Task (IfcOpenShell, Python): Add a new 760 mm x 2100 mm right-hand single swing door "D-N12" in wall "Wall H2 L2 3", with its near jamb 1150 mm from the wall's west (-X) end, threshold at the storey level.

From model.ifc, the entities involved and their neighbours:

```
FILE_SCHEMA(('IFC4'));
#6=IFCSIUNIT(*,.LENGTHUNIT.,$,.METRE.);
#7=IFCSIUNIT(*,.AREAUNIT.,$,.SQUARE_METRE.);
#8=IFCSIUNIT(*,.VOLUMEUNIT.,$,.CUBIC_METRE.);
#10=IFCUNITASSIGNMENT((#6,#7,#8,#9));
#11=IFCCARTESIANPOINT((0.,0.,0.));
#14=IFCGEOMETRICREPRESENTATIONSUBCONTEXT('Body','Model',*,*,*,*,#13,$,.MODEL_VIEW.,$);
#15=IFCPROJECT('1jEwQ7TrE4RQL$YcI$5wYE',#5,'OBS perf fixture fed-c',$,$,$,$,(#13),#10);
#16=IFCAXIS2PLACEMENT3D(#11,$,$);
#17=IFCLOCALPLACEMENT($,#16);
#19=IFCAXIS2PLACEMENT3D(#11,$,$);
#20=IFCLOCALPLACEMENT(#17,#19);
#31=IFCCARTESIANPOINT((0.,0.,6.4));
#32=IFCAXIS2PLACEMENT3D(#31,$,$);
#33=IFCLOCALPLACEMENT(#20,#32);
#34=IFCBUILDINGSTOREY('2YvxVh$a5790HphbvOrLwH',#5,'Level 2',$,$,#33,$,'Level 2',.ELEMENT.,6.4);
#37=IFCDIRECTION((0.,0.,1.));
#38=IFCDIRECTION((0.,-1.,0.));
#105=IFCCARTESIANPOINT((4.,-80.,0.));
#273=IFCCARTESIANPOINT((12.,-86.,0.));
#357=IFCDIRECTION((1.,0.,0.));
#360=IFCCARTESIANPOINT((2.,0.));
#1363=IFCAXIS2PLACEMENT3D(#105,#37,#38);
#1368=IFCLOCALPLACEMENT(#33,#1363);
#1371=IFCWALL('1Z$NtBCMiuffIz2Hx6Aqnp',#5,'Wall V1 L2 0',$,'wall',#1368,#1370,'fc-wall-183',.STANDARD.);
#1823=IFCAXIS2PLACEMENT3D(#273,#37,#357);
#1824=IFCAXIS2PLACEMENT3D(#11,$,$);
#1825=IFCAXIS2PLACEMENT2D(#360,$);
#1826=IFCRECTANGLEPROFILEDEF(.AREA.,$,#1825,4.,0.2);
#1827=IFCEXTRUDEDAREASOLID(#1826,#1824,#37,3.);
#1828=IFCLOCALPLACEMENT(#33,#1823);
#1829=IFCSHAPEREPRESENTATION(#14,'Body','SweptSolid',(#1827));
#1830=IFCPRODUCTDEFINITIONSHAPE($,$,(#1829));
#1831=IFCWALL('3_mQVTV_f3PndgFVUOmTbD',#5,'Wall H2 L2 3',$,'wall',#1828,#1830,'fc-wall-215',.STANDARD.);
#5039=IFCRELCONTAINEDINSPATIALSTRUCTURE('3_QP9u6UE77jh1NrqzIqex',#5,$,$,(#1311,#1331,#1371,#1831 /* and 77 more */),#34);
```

```python
import numpy as np
import ifcopenshell
import ifcopenshell.api.feature
import ifcopenshell.api.geometry
import ifcopenshell.api.root
import ifcopenshell.api.spatial
import ifcopenshell.geom
import ifcopenshell.util.element
import ifcopenshell.util.placement
import ifcopenshell.util.representation
import ifcopenshell.util.shape
import ifcopenshell.util.unit

model = ifcopenshell.open("model.ifc")
unit_scale = ifcopenshell.util.unit.calculate_unit_scale(model)
settings = ifcopenshell.geom.settings()


def volume(element):
    """Net volume in cubic metres, openings subtracted."""
    shape = ifcopenshell.geom.create_shape(settings, element)
    return ifcopenshell.util.shape.get_volume(shape.geometry)


wall = model.by_id(1831)
storey = ifcopenshell.util.element.get_container(wall, ifc_class="IfcBuildingStorey")
context = ifcopenshell.util.representation.get_context(model, "Model", "Body", "MODEL_VIEW")
before = volume(wall)

width, height, from_end, sill = 0.76, 2.1, 1.15, 0.0  # metres

# The wall runs along its own X axis, and the end named is its -X end.
wall_shape = ifcopenshell.geom.create_shape(settings, wall)
x, y, z = ifcopenshell.util.shape.get_vertices(wall_shape.geometry).T
start = x.min() + from_end
face, thickness = float(y.min()), float(y.max() - y.min())
wall_matrix = ifcopenshell.util.placement.get_local_placement(wall.ObjectPlacement)
level = ifcopenshell.util.placement.get_local_placement(storey.ObjectPlacement)[2, 3]


def in_wall(x, y):
    """Placement at x, y metres in the wall's axes, at sill height."""
    matrix = wall_matrix.copy()
    matrix[:, 3] = wall_matrix @ np.array([x / unit_scale, y / unit_scale, 0.0, 1.0])
    matrix[2, 3] = level + sill / unit_scale
    return matrix


# Opening: a box that overshoots both wall faces by 50 mm.
opening = ifcopenshell.api.root.create_entity(model, ifc_class="IfcOpeningElement", predefined_type="OPENING")
box = ifcopenshell.api.geometry.add_wall_representation(
    model, context=context, length=width, height=height, thickness=thickness + 0.1
)
ifcopenshell.api.geometry.assign_representation(model, product=opening, representation=box)
ifcopenshell.api.geometry.edit_object_placement(model, product=opening, matrix=in_wall(start, face - 0.05), is_si=False)
ifcopenshell.api.feature.add_feature(model, feature=opening, element=wall)

door = ifcopenshell.api.root.create_entity(model, ifc_class="IfcDoor", name="D-N12", predefined_type="DOOR")
door.OverallWidth, door.OverallHeight = width / unit_scale, height / unit_scale
door.OperationType = "SINGLE_SWING_RIGHT"
body = ifcopenshell.api.geometry.add_door_representation(
    model,
    context=context,
    overall_width=door.OverallWidth,
    overall_height=door.OverallHeight,
    operation_type="SINGLE_SWING_RIGHT",
    lining_properties={"LiningDepth": thickness / unit_scale, "ThresholdDepth": thickness / unit_scale},
)
ifcopenshell.api.geometry.assign_representation(model, product=door, representation=body)
ifcopenshell.api.spatial.assign_container(model, products=[door], relating_structure=storey)
ifcopenshell.api.feature.add_filling(model, opening=opening, element=door)

# The lining spans the wall, so the door starts at the wall face.
ifcopenshell.api.geometry.edit_object_placement(model, product=door, matrix=in_wall(start, face), is_si=False)

after = volume(wall)

print(f"wall volume {before:.3f} -> {after:.3f} m3")

model.write("model-out.ifc")
```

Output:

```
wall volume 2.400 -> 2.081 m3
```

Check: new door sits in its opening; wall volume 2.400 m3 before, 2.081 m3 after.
